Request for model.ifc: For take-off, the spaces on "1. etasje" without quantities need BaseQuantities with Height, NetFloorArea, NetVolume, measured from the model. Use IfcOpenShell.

First a look at what the model holds.

```python
import ifcopenshell
import ifcopenshell.util.element
import ifcopenshell.util.unit

model = ifcopenshell.open("model.ifc")
print(model.schema)
for unit_type in ("LENGTHUNIT", "AREAUNIT", "VOLUMEUNIT"):
    print(unit_type, ifcopenshell.util.unit.calculate_unit_scale(model, unit_type))
storey = next(s for s in model.by_type("IfcBuildingStorey") if s.Name == "1. etasje")
spaces = [e for e in ifcopenshell.util.element.get_decomposition(storey) if e.is_a("IfcSpace")]
for e in sorted(spaces, key=lambda e: e.id()):
    print(e.id(), e.is_a(), e.Name, list(ifcopenshell.util.element.get_psets(e, qtos_only=True)), sep=" | ")
```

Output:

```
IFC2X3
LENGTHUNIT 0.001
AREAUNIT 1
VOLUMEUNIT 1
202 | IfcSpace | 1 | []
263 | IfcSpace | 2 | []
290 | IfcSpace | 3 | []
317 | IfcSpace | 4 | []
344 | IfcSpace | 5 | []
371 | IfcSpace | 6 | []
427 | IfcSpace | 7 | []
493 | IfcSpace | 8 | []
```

```python
import ifcopenshell
import ifcopenshell.api.pset
import ifcopenshell.geom
import ifcopenshell.util.element
import ifcopenshell.util.shape
import ifcopenshell.util.unit

model = ifcopenshell.open("model.ifc")
unit_scale = ifcopenshell.util.unit.calculate_unit_scale(model)
area_scale = ifcopenshell.util.unit.calculate_unit_scale(model, "AREAUNIT")
volume_scale = ifcopenshell.util.unit.calculate_unit_scale(model, "VOLUMEUNIT")
settings = ifcopenshell.geom.settings()

storey = next(s for s in model.by_type("IfcBuildingStorey") if s.Name == "1. etasje")
spaces = [e for e in ifcopenshell.util.element.get_decomposition(storey) if e.is_a("IfcSpace")]

for e in sorted(spaces, key=lambda e: e.id()):
    if ifcopenshell.util.element.get_psets(e, qtos_only=True, should_inherit=False):
        continue
    # Geometry comes back in metres, in the element's own axes.
    shape = ifcopenshell.geom.create_shape(settings, e)
    values = {
        "Height": ifcopenshell.util.shape.get_z(shape.geometry) / unit_scale,
        "NetFloorArea": ifcopenshell.util.shape.get_footprint_area(shape.geometry) / area_scale,
        "NetVolume": ifcopenshell.util.shape.get_volume(shape.geometry) / volume_scale,
    }
    qto = ifcopenshell.api.pset.add_qto(model, product=e, name="BaseQuantities")
    ifcopenshell.api.pset.edit_qto(model, qto=qto, properties=values)
    print(e.id(), {k: round(v, 3) for k, v in values.items()})

model.write("model_rev.ifc")
```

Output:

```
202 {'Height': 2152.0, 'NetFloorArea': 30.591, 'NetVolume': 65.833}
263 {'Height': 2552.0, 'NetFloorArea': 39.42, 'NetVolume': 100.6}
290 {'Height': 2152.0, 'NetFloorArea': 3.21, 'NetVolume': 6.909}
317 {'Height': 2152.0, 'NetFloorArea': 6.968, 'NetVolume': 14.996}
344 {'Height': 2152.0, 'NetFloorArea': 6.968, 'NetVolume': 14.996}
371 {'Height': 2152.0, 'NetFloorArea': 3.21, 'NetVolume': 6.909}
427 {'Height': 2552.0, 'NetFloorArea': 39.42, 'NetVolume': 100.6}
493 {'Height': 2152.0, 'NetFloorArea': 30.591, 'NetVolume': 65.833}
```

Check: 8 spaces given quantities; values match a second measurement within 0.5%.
